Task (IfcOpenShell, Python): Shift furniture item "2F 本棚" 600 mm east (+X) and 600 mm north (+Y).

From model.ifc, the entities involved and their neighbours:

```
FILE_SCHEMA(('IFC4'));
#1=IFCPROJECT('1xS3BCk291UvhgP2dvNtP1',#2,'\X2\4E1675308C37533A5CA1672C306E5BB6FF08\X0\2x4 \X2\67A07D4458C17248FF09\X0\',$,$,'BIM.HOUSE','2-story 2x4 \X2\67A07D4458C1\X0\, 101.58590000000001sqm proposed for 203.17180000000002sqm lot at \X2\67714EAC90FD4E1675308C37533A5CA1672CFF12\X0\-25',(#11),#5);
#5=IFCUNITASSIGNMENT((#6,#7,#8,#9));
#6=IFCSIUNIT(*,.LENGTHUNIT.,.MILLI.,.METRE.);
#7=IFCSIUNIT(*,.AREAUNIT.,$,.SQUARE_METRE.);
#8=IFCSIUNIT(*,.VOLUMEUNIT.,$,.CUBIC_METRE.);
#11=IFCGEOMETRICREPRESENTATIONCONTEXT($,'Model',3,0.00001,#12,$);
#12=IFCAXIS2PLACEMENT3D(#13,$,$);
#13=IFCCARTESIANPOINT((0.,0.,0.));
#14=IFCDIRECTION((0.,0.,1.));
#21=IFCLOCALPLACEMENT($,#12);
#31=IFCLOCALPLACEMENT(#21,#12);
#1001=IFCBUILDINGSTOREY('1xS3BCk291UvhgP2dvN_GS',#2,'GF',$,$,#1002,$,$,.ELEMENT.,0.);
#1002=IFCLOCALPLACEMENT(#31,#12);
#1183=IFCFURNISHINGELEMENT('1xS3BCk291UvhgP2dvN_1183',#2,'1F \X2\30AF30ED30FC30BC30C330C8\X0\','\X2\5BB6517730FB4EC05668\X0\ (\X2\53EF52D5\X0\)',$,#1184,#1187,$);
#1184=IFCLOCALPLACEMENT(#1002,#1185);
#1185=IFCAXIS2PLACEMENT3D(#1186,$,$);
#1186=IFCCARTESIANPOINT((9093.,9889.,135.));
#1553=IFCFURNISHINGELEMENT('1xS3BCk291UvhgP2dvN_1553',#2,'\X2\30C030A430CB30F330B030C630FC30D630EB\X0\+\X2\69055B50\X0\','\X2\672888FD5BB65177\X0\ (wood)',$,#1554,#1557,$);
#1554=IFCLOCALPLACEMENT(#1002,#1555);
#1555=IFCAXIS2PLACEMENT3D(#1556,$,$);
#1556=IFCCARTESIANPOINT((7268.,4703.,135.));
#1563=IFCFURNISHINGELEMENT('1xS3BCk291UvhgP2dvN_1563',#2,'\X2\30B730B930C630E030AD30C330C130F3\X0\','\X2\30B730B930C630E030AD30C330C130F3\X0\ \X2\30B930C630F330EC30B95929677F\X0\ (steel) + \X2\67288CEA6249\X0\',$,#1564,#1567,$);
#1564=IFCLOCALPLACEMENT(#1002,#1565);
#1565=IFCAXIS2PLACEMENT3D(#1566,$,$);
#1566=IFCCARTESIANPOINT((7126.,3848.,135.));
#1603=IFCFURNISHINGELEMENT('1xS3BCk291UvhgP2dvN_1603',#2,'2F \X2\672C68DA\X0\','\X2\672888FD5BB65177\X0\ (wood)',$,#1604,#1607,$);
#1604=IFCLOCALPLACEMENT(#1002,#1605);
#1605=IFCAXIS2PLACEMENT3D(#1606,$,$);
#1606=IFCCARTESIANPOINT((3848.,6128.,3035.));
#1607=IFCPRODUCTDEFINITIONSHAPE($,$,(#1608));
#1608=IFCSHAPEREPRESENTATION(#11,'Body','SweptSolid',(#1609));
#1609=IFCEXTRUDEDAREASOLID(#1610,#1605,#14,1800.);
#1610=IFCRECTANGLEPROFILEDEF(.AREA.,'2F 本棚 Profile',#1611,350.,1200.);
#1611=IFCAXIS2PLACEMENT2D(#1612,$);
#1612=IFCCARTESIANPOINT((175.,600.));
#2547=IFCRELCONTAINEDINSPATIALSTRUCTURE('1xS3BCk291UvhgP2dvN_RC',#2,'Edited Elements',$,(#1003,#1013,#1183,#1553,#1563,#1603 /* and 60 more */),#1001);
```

```python
import ifcopenshell
import ifcopenshell.api.geometry
import ifcopenshell.util.placement

model = ifcopenshell.open("model.ifc")

item = model.by_guid("1xS3BCk291UvhgP2dvN_1603")
matrix = ifcopenshell.util.placement.get_local_placement(item.ObjectPlacement)
matrix[0, 3] += 600.0
matrix[1, 3] += 600.0
ifcopenshell.api.geometry.edit_object_placement(model, product=item, matrix=matrix, is_si=False)

print(ifcopenshell.util.placement.get_local_placement(item.ObjectPlacement).round(3) + 0.0)

model.write("model_edited.ifc")
```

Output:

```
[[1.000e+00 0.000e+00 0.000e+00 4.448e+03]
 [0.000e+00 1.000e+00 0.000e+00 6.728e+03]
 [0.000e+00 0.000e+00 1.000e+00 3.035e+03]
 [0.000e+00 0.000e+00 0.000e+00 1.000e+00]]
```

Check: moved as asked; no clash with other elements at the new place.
